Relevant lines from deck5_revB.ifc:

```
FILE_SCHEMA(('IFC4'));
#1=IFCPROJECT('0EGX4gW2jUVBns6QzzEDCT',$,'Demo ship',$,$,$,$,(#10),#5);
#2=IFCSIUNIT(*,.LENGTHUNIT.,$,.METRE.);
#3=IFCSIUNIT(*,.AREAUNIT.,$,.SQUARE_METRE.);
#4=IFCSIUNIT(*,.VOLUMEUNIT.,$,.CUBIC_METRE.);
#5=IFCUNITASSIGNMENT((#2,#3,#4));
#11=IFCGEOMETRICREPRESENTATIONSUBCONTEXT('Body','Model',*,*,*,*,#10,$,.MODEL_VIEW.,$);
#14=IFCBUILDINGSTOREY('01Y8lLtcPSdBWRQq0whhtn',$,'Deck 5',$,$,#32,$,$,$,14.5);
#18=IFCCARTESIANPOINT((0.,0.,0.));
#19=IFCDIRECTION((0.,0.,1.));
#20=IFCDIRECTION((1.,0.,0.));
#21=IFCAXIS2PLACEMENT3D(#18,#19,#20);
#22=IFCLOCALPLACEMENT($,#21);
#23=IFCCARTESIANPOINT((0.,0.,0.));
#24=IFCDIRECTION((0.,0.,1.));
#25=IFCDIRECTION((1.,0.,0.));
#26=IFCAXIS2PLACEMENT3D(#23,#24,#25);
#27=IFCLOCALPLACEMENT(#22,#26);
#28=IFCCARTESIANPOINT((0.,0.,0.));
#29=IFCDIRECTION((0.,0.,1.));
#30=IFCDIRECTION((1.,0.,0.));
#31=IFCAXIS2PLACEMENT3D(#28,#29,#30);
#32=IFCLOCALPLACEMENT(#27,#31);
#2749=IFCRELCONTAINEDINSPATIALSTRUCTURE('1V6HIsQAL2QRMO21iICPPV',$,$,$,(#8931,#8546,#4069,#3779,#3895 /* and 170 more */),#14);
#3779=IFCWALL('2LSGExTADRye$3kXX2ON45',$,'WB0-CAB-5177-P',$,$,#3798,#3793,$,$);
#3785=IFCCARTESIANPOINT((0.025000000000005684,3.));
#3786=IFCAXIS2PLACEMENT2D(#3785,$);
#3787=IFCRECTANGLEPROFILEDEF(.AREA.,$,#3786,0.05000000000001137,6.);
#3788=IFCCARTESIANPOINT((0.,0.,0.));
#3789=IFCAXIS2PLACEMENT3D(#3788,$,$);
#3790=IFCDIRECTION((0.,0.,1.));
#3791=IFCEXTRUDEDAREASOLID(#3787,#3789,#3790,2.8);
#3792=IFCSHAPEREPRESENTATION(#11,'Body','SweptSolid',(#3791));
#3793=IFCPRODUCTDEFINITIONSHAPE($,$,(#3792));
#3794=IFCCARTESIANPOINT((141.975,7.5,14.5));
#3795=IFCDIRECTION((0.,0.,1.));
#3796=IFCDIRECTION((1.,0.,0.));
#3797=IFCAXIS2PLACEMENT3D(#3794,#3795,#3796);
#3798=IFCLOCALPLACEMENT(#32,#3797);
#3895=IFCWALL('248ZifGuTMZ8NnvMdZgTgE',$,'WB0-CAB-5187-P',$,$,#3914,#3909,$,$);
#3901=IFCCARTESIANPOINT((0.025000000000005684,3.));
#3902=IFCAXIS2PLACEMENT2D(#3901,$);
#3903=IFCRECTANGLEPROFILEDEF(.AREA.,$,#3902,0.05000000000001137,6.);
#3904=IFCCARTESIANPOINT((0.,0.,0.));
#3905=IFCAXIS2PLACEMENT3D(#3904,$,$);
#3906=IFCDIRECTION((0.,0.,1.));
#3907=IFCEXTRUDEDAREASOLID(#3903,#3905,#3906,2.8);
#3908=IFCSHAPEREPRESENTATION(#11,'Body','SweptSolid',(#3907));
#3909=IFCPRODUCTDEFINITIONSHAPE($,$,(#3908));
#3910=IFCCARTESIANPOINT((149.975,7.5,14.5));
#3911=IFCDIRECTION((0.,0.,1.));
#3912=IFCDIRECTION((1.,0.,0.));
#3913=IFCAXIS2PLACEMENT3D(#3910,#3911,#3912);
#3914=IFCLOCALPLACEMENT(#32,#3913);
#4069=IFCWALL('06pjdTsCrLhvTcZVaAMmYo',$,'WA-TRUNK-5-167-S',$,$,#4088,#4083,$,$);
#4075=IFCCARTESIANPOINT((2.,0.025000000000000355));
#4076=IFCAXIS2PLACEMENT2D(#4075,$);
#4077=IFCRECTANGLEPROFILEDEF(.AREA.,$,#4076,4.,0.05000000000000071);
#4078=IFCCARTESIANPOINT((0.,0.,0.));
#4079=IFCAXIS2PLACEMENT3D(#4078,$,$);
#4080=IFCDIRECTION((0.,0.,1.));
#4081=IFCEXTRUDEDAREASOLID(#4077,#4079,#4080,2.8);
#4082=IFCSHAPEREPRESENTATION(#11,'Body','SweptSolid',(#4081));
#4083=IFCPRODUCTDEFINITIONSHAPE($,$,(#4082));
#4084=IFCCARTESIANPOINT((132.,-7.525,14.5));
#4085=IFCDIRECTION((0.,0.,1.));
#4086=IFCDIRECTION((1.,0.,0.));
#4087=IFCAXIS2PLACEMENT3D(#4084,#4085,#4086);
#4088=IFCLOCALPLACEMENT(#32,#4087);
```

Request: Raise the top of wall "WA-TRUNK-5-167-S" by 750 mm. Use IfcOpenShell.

```python
import ifcopenshell
import ifcopenshell.geom
import ifcopenshell.util.representation
import ifcopenshell.util.shape
import ifcopenshell.util.unit

model = ifcopenshell.open("deck5_revB.ifc")
unit_scale = ifcopenshell.util.unit.calculate_unit_scale(model)
settings = ifcopenshell.geom.settings()


def volume(element):
    """Net volume in cubic metres, openings subtracted."""
    shape = ifcopenshell.geom.create_shape(settings, element)
    return ifcopenshell.util.shape.get_volume(shape.geometry)


wall = model.by_guid("06pjdTsCrLhvTcZVaAMmYo")
before = volume(wall)

body = ifcopenshell.util.representation.get_representation(wall, "Model", "Body")
solid = body.Items[0]
old_height = solid.Depth
solid.Depth += 0.75 / unit_scale
after = volume(wall)

print(f"height {old_height:g} -> {solid.Depth:g}, volume {before:.3f} -> {after:.3f} m3")

model.write("deck5_revB_v2.ifc")
```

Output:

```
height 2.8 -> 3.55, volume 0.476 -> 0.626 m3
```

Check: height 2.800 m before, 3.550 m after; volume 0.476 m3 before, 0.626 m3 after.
